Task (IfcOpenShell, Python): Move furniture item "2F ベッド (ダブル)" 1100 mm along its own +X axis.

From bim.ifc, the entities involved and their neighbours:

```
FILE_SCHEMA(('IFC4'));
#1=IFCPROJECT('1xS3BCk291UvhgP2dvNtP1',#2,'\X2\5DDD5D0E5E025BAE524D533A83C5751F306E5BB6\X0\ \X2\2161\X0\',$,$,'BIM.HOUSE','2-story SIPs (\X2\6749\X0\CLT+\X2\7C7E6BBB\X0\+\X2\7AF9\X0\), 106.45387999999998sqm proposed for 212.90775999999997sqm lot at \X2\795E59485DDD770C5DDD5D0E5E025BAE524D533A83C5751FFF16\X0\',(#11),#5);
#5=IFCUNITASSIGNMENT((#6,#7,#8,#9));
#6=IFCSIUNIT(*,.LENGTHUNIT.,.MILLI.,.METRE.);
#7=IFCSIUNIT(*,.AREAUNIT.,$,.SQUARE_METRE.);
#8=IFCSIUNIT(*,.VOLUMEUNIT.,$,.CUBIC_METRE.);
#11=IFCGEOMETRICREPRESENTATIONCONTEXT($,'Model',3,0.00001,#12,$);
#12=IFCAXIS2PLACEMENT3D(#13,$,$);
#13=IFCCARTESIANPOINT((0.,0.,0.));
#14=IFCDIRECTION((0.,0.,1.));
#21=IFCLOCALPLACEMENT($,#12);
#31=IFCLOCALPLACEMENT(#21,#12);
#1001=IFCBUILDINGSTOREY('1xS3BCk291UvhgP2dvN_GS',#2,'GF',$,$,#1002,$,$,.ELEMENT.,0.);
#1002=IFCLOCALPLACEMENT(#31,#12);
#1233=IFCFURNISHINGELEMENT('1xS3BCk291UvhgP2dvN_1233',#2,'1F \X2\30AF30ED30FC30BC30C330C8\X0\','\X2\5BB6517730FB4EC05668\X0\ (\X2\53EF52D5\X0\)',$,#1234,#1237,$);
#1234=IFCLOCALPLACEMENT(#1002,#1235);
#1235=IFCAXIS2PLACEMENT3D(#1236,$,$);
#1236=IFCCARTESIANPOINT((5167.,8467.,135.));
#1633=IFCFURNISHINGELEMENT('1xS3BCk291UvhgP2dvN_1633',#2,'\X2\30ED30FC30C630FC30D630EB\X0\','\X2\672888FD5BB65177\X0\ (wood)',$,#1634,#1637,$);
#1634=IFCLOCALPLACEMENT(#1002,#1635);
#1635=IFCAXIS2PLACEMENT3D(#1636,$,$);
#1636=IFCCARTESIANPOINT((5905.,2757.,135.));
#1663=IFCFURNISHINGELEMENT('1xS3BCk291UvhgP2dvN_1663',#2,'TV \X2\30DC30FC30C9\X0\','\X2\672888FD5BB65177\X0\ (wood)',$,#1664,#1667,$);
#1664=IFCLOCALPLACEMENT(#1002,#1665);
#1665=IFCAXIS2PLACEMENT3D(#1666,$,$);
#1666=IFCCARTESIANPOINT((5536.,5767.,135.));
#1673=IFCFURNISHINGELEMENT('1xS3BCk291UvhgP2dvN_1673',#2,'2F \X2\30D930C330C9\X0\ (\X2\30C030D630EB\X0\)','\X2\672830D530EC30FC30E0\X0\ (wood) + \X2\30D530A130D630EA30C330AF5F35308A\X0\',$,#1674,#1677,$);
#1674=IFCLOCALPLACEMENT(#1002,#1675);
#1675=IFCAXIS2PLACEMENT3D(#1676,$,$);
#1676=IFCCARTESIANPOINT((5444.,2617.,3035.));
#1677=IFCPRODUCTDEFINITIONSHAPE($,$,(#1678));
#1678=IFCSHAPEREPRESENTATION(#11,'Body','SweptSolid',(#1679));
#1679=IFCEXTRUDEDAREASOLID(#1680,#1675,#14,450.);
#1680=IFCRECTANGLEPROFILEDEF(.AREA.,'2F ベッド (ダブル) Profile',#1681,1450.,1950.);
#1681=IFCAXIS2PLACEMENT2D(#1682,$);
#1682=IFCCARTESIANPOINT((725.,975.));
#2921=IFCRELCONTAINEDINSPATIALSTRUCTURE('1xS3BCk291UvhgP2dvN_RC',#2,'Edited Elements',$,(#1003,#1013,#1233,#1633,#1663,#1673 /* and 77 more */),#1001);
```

```python
import ifcopenshell
import ifcopenshell.api.geometry
import ifcopenshell.util.placement

model = ifcopenshell.open("bim.ifc")

item = model.by_guid("1xS3BCk291UvhgP2dvN_1673")
matrix = ifcopenshell.util.placement.get_local_placement(item.ObjectPlacement)
matrix[:3, 3] += matrix[:3, 0] * 1100.0
ifcopenshell.api.geometry.edit_object_placement(model, product=item, matrix=matrix, is_si=False)

print(ifcopenshell.util.placement.get_local_placement(item.ObjectPlacement).round(3) + 0.0)

model.write("bim-out.ifc")
```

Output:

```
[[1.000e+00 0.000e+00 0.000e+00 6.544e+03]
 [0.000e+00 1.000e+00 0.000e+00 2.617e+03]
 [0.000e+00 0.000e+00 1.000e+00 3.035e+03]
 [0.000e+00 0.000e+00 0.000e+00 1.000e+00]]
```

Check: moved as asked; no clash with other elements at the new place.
